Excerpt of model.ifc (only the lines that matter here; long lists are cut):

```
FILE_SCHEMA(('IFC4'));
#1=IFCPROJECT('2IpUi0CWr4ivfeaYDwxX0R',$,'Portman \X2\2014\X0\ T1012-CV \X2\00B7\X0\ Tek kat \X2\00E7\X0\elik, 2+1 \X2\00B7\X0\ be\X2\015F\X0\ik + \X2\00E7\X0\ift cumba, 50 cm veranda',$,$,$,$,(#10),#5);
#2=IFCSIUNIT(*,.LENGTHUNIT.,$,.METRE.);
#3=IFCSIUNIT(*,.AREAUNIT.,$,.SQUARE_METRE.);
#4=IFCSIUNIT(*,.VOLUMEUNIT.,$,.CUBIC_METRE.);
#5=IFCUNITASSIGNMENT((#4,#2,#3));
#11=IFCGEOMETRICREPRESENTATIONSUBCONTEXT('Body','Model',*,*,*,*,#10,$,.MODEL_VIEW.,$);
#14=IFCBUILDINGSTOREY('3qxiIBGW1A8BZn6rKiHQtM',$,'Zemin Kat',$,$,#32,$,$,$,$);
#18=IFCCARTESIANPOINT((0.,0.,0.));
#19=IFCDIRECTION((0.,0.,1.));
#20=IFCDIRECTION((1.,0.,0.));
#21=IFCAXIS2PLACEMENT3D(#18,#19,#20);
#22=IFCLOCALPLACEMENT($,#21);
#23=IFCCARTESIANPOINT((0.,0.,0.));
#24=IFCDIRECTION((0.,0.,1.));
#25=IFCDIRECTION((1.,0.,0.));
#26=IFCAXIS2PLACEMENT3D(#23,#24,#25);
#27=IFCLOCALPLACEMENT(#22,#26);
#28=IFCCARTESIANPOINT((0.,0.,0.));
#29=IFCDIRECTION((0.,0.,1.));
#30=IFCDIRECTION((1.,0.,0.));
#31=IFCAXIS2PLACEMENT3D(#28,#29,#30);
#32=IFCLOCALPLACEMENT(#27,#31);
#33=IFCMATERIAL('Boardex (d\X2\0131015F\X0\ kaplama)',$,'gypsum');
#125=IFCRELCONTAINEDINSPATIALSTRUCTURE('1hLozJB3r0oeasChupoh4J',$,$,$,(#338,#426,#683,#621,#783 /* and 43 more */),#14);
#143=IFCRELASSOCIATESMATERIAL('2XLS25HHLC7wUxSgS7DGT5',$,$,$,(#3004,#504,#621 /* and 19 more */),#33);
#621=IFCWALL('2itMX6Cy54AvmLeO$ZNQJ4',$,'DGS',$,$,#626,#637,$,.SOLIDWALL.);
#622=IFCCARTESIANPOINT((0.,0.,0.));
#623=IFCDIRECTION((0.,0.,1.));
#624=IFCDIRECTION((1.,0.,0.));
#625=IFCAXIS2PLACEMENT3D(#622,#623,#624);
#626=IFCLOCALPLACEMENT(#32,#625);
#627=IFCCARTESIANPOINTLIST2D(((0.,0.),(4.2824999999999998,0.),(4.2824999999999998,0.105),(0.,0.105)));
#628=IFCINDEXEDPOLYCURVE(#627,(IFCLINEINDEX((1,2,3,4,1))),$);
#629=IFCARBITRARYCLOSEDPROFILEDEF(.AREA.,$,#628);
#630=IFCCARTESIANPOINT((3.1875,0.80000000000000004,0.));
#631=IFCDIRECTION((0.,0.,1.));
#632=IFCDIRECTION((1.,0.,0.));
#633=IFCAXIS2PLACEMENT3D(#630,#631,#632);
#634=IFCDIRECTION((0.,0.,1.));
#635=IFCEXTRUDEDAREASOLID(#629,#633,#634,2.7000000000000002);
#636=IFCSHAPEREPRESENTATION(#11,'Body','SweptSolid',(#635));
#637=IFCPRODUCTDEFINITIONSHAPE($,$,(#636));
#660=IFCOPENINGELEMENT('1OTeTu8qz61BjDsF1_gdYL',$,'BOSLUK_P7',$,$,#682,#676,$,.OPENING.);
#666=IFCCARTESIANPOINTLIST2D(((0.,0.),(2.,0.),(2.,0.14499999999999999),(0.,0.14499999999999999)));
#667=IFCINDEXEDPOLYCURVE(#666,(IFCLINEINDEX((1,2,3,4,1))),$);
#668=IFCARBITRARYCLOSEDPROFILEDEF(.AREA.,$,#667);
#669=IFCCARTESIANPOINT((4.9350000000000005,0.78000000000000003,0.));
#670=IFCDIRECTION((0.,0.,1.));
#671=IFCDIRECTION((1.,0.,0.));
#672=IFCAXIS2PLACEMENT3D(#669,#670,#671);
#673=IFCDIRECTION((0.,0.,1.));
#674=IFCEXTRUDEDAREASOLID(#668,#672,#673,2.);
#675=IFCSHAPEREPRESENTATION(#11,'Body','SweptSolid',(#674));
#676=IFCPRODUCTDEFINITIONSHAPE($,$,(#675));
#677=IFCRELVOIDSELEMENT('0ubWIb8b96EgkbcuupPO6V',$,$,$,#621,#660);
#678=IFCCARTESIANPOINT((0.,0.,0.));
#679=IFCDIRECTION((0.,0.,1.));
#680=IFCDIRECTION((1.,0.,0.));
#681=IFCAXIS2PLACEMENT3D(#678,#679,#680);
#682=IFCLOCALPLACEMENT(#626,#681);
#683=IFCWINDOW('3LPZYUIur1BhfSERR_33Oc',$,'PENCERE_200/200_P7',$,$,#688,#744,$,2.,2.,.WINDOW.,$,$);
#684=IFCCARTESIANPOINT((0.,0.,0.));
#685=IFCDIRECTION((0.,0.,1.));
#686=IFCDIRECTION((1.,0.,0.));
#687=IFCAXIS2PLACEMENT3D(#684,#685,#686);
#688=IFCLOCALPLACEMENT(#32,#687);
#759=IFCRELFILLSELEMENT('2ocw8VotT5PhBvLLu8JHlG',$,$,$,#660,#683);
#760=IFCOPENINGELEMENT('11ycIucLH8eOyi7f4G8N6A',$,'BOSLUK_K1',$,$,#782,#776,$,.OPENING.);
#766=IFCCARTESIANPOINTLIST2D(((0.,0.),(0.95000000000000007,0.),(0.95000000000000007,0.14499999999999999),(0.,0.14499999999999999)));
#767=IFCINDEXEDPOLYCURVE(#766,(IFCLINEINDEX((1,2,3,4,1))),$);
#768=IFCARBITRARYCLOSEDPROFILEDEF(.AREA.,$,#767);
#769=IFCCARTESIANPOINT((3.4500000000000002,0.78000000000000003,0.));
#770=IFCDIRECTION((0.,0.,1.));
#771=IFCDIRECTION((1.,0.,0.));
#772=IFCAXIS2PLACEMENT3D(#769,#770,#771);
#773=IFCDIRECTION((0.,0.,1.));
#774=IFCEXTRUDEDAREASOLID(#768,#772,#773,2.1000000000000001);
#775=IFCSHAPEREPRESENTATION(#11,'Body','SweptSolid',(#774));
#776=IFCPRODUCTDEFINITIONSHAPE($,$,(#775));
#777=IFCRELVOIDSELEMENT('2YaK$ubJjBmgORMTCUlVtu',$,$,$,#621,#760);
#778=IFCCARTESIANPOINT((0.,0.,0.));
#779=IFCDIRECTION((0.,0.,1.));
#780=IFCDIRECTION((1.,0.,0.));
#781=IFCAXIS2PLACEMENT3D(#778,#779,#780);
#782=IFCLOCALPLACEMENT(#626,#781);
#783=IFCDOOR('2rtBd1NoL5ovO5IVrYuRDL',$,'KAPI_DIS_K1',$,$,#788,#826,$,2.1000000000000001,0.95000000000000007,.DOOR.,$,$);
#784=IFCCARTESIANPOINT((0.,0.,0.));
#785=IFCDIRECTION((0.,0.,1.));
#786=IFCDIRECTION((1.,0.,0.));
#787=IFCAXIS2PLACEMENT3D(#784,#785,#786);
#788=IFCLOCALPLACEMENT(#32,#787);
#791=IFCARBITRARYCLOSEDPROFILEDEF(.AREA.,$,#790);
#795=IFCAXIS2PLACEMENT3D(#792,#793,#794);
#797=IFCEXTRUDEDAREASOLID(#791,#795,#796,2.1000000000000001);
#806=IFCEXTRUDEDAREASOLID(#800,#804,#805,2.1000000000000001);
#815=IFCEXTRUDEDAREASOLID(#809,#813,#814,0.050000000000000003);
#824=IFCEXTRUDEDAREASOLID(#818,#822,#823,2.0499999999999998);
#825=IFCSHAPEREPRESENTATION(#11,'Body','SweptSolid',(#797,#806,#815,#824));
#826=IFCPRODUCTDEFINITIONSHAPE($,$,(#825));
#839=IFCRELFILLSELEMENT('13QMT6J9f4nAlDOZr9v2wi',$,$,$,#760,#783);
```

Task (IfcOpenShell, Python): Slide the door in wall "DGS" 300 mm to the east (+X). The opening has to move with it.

```python
import ifcopenshell
import ifcopenshell.api.geometry
import ifcopenshell.util.placement
import ifcopenshell.util.unit

model = ifcopenshell.open("model.ifc")
unit_scale = ifcopenshell.util.unit.calculate_unit_scale(model)

door = model.by_guid("2rtBd1NoL5ovO5IVrYuRDL")
opening = door.FillsVoids[0].RelatingOpeningElement
wall = opening.VoidsElements[0].RelatingBuildingElement

wall_matrix = ifcopenshell.util.placement.get_local_placement(wall.ObjectPlacement)
shift = wall_matrix[:3, 0] * 0.3 / unit_scale
before = ifcopenshell.util.placement.get_local_placement(door.ObjectPlacement)[:3, 3].copy()

# The door is not placed relative to its opening, so move both.
for product in (opening, door):
    matrix = ifcopenshell.util.placement.get_local_placement(product.ObjectPlacement)
    matrix[:3, 3] += shift
    ifcopenshell.api.geometry.edit_object_placement(model, product=product, matrix=matrix, is_si=False)

after = ifcopenshell.util.placement.get_local_placement(door.ObjectPlacement)[:3, 3]
print("door moved by", (after - before).round(3) + 0.0)

model.write("model_rev.ifc")
```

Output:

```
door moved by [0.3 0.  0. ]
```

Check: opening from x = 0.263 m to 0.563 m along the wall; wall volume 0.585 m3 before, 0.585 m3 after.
